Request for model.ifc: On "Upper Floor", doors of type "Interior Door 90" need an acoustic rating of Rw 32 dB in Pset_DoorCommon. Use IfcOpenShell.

First a look at what the model holds.

```python
import ifcopenshell
import ifcopenshell.util.element

model = ifcopenshell.open("model.ifc")
print(model.schema)
storey = next(s for s in model.by_type("IfcBuildingStorey") if s.Name == "Upper Floor")
doors = [e for e in ifcopenshell.util.element.get_decomposition(storey) if e.is_a("IfcDoor")]
seen = {}
for e in doors:
    element_type = ifcopenshell.util.element.get_type(e)
    key = (element_type.Name if element_type != e and element_type else None, ifcopenshell.util.element.get_pset(e, "Pset_DoorCommon", "AcousticRating"))
    seen[key] = seen.get(key, 0) + 1
for (name, value), count in sorted(seen.items(), key=str):
    print(count, "x", name, "|", value)
```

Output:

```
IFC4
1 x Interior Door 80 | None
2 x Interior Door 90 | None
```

```python
import ifcopenshell
import ifcopenshell.api.pset
import ifcopenshell.util.element

model = ifcopenshell.open("model.ifc")

storey = next(s for s in model.by_type("IfcBuildingStorey") if s.Name == "Upper Floor")
doors = [e for e in ifcopenshell.util.element.get_decomposition(storey) if e.is_a("IfcDoor")]

count = 0
for e in doors:
    element_type = ifcopenshell.util.element.get_type(e)
    if element_type in (None, e) or element_type.Name != "Interior Door 90":
        continue
    # add_pset returns the element's existing set when there is one.
    pset = ifcopenshell.api.pset.add_pset(model, product=e, name="Pset_DoorCommon")
    ifcopenshell.api.pset.edit_pset(model, pset=pset, properties={"AcousticRating": "Rw 32 dB"})
    count += 1

print(count, "doors updated")

model.write("model_edited.ifc")
```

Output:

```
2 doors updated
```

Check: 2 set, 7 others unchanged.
